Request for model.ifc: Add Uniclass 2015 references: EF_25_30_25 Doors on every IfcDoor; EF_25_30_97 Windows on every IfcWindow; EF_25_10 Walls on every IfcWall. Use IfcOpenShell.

First a look at what the model holds.

```python
import ifcopenshell

model = ifcopenshell.open("model.ifc")
print(model.schema)
print("classifications:", [c.Name for c in model.by_type("IfcClassification")])
for ifc_class in ("IfcDoor", "IfcRoof", "IfcStair", "IfcWall", "IfcWindow"):
    print(ifc_class, len(model.by_type(ifc_class)))
```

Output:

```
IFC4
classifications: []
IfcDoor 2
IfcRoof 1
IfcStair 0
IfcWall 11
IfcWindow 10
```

```python
import ifcopenshell
import ifcopenshell.api.classification

model = ifcopenshell.open("model.ifc")

system = ifcopenshell.api.classification.add_classification(model, classification="Uniclass 2015")

codes = {
    "IfcDoor": ("EF_25_30_25", "Doors"),
    "IfcWindow": ("EF_25_30_97", "Windows"),
    "IfcWall": ("EF_25_10", "Walls"),
}
for ifc_class, (code, name) in codes.items():
    products = model.by_type(ifc_class)
    ifcopenshell.api.classification.add_reference(
        model, products=products, classification=system, identification=code, name=name
    )
    print(code, len(products))

model.write("model-out.ifc")
```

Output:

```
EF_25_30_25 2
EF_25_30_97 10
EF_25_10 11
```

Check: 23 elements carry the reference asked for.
